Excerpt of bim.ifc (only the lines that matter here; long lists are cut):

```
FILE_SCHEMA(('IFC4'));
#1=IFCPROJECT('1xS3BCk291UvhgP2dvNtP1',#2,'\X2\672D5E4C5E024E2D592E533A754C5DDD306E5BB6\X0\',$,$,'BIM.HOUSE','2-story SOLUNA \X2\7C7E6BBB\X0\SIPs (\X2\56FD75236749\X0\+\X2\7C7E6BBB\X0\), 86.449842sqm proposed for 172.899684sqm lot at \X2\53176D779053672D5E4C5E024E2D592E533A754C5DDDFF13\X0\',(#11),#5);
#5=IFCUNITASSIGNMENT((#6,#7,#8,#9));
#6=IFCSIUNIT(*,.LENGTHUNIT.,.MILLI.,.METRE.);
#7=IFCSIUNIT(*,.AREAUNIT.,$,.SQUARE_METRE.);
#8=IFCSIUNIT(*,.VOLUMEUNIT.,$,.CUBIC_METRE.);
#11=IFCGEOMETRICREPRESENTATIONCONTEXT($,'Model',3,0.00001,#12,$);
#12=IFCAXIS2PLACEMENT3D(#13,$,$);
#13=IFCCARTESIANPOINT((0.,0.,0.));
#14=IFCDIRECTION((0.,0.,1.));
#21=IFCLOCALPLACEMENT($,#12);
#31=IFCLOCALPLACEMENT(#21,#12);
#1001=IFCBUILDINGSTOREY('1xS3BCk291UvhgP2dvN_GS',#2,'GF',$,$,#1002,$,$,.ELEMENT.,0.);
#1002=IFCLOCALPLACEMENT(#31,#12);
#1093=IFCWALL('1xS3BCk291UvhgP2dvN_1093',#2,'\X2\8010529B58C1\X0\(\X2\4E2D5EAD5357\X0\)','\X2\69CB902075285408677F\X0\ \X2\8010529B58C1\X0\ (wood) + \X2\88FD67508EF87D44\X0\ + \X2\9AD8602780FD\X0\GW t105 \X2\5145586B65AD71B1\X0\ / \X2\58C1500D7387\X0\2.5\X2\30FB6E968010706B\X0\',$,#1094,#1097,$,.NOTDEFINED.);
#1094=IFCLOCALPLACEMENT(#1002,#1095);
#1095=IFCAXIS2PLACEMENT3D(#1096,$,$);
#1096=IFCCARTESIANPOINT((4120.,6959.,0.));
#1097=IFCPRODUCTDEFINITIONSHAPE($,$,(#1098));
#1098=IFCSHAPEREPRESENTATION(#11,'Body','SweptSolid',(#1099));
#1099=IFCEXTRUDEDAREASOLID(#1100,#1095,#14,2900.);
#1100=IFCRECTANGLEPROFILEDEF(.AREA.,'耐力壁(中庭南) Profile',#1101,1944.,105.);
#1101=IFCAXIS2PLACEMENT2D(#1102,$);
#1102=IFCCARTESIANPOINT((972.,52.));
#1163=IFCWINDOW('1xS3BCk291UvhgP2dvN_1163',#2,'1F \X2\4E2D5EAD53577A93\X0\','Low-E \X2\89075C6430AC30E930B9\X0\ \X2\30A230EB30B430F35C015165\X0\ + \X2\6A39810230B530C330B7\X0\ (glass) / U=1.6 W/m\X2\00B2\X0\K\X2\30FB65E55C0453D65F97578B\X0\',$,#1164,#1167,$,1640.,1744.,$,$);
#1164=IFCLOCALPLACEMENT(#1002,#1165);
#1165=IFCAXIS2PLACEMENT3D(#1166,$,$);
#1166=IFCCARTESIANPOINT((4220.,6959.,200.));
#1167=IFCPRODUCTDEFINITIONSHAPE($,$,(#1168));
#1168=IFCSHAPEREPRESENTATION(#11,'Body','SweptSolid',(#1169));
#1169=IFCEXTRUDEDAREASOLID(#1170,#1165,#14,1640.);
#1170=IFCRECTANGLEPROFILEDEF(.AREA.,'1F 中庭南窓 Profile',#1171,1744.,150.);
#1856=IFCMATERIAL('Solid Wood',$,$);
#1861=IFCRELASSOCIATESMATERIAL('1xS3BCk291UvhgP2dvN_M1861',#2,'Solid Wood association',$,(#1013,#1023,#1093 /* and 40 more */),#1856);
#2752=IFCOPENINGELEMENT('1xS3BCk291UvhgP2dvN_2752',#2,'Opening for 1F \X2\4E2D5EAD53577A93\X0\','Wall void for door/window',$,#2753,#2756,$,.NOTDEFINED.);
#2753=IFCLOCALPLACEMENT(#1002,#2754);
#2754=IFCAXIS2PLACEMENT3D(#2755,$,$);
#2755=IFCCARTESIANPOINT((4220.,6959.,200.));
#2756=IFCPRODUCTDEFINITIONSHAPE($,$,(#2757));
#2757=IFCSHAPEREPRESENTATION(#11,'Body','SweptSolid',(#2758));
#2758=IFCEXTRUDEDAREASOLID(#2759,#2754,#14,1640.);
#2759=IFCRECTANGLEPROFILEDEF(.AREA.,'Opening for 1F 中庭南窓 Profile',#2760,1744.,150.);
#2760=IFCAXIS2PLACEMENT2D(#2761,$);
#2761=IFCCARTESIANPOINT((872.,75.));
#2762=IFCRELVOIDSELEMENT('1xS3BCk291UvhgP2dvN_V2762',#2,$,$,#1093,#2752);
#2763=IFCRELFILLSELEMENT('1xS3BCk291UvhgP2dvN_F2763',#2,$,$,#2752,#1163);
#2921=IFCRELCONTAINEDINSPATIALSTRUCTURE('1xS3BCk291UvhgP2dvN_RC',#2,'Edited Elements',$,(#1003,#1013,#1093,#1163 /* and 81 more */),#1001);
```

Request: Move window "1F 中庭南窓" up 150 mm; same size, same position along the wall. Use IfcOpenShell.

```python
import numpy as np
import ifcopenshell
import ifcopenshell.api.geometry
import ifcopenshell.util.placement
import ifcopenshell.util.unit

model = ifcopenshell.open("bim.ifc")
unit_scale = ifcopenshell.util.unit.calculate_unit_scale(model)

window = model.by_id(1163)
opening = window.FillsVoids[0].RelatingOpeningElement
dz = 0.15 / unit_scale

shift = np.array([0.0, 0.0, dz])
# The window is not placed relative to its opening, so move both.
for product in (opening, window):
    matrix = ifcopenshell.util.placement.get_local_placement(product.ObjectPlacement)
    matrix[:3, 3] += shift
    ifcopenshell.api.geometry.edit_object_placement(model, product=product, matrix=matrix, is_si=False)

print(f"moved by {dz * unit_scale:+.3f} m")

model.write("bim_rev.ifc")
```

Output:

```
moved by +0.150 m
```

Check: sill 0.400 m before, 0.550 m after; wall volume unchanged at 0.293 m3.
